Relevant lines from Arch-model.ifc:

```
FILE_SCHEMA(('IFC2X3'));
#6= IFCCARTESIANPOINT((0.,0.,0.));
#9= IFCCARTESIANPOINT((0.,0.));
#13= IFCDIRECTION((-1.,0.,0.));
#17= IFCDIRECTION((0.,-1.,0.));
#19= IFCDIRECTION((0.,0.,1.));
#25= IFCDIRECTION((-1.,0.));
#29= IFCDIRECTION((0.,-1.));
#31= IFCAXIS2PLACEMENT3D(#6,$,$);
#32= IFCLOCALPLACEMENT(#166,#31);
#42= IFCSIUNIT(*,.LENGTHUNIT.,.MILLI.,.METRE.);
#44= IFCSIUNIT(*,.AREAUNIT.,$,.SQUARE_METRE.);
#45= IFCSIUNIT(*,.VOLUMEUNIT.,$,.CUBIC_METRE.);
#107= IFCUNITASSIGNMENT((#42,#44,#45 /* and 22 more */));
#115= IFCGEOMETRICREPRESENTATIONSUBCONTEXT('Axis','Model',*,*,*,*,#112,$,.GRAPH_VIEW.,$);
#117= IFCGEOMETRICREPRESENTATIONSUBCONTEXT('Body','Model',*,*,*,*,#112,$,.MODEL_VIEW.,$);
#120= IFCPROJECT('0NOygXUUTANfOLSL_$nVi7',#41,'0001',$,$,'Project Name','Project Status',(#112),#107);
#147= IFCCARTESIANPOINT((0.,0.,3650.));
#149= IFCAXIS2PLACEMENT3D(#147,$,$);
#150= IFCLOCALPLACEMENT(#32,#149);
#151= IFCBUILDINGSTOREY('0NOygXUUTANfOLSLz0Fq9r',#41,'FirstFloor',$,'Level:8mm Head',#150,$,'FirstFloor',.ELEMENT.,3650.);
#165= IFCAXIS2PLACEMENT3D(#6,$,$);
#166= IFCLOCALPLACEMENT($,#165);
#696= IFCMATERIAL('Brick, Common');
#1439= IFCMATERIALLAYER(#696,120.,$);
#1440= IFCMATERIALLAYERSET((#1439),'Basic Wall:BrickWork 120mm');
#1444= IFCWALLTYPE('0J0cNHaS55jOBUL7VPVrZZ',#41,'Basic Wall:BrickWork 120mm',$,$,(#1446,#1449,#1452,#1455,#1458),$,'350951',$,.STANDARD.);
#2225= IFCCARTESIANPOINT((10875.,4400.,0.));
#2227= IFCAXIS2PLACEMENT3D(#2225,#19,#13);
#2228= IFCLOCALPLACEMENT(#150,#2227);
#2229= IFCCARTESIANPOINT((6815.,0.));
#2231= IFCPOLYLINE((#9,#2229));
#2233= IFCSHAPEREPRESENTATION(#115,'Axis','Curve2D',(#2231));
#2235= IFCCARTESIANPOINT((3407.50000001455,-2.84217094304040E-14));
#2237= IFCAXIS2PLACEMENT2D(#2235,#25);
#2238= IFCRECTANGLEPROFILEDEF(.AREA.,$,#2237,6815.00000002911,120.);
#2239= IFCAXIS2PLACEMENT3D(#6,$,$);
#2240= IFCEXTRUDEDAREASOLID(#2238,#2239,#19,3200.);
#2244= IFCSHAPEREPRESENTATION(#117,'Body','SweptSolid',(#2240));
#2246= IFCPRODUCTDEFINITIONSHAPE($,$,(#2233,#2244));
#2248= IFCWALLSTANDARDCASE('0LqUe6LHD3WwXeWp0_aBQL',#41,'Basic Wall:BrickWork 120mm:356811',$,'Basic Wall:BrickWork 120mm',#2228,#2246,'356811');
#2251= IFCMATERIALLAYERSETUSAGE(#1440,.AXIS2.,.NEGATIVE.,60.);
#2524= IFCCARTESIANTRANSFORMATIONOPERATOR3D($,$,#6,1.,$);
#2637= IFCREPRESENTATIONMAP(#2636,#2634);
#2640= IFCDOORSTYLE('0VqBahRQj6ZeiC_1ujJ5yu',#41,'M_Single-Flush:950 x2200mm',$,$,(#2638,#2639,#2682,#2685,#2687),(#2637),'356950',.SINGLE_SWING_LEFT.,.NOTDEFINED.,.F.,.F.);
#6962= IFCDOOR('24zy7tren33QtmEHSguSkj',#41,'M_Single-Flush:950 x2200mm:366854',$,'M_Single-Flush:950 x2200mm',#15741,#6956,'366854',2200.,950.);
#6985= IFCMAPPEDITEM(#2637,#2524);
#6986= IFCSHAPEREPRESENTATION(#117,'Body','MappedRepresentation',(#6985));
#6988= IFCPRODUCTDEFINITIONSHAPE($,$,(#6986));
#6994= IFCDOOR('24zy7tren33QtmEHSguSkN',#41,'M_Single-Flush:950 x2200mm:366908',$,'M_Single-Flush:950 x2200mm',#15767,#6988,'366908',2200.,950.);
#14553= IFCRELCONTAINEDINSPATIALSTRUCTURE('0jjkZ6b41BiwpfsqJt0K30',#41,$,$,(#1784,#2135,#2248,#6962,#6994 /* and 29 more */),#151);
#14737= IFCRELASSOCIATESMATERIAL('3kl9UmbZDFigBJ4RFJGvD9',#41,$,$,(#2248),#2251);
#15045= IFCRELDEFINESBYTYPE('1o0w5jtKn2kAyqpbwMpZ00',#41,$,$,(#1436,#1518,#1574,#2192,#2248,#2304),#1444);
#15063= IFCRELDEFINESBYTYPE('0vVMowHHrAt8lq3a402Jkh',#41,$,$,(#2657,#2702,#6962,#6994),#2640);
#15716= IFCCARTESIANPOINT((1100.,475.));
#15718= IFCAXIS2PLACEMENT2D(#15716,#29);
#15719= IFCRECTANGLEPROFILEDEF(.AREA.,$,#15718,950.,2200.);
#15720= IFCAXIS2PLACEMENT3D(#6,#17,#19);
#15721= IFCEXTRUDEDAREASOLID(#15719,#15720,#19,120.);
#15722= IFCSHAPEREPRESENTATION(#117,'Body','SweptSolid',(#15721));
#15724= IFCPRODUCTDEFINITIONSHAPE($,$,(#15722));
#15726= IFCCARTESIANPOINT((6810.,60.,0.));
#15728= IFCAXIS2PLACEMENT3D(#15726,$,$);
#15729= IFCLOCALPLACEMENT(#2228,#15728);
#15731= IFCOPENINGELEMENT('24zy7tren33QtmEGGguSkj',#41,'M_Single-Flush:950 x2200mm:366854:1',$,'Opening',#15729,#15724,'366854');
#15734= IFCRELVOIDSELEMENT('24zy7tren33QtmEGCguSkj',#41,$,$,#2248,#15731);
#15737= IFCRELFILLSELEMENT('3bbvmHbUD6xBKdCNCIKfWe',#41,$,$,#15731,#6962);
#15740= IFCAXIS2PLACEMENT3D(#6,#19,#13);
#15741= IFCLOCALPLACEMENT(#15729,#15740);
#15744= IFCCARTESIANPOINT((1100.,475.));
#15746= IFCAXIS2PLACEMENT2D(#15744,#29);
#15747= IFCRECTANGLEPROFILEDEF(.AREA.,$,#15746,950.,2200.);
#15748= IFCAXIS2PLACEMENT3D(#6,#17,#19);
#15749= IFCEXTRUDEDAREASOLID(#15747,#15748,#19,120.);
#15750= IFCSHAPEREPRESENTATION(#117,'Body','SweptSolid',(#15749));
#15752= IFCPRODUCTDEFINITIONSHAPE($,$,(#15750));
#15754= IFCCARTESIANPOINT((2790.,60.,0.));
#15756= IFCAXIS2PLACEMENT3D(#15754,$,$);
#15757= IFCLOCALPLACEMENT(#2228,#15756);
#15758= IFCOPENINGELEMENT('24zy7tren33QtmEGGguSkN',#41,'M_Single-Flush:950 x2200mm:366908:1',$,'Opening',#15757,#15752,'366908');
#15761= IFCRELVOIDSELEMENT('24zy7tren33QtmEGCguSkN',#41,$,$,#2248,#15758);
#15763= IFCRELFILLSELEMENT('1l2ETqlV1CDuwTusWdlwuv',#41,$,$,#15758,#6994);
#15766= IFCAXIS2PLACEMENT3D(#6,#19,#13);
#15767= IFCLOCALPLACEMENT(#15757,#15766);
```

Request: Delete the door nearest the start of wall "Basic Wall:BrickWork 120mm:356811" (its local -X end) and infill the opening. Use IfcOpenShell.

```python
import ifcopenshell
import ifcopenshell.api.feature
import ifcopenshell.api.root
import ifcopenshell.geom
import ifcopenshell.util.shape

model = ifcopenshell.open("Arch-model.ifc")
settings = ifcopenshell.geom.settings()


def volume(element):
    """Net volume in cubic metres, openings subtracted."""
    shape = ifcopenshell.geom.create_shape(settings, element)
    return ifcopenshell.util.shape.get_volume(shape.geometry)


door = model.by_guid("24zy7tren33QtmEHSguSkN")
opening = door.FillsVoids[0].RelatingOpeningElement
wall = opening.VoidsElements[0].RelatingBuildingElement
before = volume(wall)

ifcopenshell.api.root.remove_product(model, product=door)
ifcopenshell.api.feature.remove_feature(model, feature=opening)

after = volume(wall)

print(f"wall volume {before:.3f} -> {after:.3f} m3")

model.write("Arch-model_updated.ifc")
```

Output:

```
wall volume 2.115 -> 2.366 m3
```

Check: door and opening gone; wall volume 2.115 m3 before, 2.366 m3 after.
